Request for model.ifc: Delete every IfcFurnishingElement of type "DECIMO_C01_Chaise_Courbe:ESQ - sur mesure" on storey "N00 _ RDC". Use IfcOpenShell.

First a look at what the model holds.

```python
import ifcopenshell
import ifcopenshell.util.element

model = ifcopenshell.open("model.ifc")
print(model.schema)
storey = next(s for s in model.by_type("IfcBuildingStorey") if s.Name == "N00 _ RDC")
furniture = [e for e in ifcopenshell.util.element.get_decomposition(storey) if e.is_a("IfcFurnishingElement")]
seen = {}
for e in furniture:
    element_type = ifcopenshell.util.element.get_type(e)
    name = element_type.Name if element_type not in (None, e) else None
    seen[name] = seen.get(name, 0) + 1
for name, count in sorted(seen.items(), key=str):
    print(count, "x", name)
```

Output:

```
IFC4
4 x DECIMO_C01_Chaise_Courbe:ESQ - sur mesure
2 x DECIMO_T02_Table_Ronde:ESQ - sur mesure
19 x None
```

```python
import ifcopenshell
import ifcopenshell.api.root
import ifcopenshell.util.element

model = ifcopenshell.open("model.ifc")

storey = next(s for s in model.by_type("IfcBuildingStorey") if s.Name == "N00 _ RDC")
furniture = [e for e in ifcopenshell.util.element.get_decomposition(storey) if e.is_a("IfcFurnishingElement")]
targets = [e for e in furniture if (t := ifcopenshell.util.element.get_type(e)) not in (None, e) and t.Name == "DECIMO_C01_Chaise_Courbe:ESQ - sur mesure"]

for e in targets:
    ifcopenshell.api.root.remove_product(model, product=e)
print(len(targets), "removed")

model.write("model-out.ifc")
```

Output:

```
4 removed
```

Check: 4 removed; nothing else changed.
